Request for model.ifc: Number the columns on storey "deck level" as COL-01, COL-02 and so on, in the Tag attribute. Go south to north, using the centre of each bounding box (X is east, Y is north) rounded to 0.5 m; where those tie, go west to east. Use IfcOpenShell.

First a look at what the model holds.

```python
import ifcopenshell
import ifcopenshell.util.element
import ifcopenshell.util.placement

model = ifcopenshell.open("model.ifc")
print(model.schema)
storey = next(s for s in model.by_type("IfcBuildingStorey") if s.Name == "deck level")
columns = [e for e in ifcopenshell.util.element.get_decomposition(storey) if e.is_a("IfcColumn")]
for e in sorted(columns, key=lambda e: e.id()):
    origin = ifcopenshell.util.placement.get_local_placement(e.ObjectPlacement)[:3, 3]
    print(e.id(), e.Tag, e.Name, origin.round(2) + 0.0, sep=" | ")
```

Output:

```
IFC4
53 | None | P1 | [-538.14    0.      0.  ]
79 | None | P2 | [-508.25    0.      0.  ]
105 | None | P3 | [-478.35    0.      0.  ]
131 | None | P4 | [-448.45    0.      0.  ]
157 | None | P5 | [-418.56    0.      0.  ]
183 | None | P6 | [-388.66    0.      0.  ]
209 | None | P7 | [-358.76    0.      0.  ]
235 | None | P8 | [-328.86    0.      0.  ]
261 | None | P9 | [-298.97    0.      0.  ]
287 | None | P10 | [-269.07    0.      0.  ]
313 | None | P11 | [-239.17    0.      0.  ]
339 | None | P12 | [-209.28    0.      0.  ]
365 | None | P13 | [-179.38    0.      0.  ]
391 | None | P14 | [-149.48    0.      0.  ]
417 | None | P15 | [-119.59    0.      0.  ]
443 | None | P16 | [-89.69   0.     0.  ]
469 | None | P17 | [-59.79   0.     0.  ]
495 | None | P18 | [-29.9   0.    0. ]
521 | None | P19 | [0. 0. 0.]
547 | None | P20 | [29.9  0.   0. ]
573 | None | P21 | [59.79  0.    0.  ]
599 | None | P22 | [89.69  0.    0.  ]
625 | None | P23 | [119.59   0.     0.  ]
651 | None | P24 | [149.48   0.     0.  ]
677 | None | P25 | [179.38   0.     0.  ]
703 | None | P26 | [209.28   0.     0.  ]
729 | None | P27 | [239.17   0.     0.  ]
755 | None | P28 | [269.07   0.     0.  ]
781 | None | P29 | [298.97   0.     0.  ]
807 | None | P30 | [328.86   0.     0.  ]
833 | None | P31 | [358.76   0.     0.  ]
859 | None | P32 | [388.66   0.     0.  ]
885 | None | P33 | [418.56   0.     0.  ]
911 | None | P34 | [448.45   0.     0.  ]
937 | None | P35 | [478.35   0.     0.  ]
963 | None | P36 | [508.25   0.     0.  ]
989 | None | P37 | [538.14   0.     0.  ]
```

```python
import ifcopenshell
import ifcopenshell.geom
import ifcopenshell.util.element
import ifcopenshell.util.shape

model = ifcopenshell.open("model.ifc")
settings = ifcopenshell.geom.settings()
settings.set("use-world-coords", True)


def centre(element):
    shape = ifcopenshell.geom.create_shape(settings, element)
    return ifcopenshell.util.shape.get_bbox_centroid(shape.geometry)


storey = next(s for s in model.by_type("IfcBuildingStorey") if s.Name == "deck level")
columns = [e for e in ifcopenshell.util.element.get_decomposition(storey) if e.is_a("IfcColumn")]

# Insertion points can sit at a corner or the storey origin, so sort by the geometry (in metres).
centres = {e: centre(e) for e in columns}
columns.sort(key=lambda e: (round(centres[e][1] / 0.5), centres[e][0]))

for i, e in enumerate(columns, start=1):
    number = f"COL-{i:02d}"
    e.Tag = number
    print(e.id(), number)

model.write("model_rev.ifc")
```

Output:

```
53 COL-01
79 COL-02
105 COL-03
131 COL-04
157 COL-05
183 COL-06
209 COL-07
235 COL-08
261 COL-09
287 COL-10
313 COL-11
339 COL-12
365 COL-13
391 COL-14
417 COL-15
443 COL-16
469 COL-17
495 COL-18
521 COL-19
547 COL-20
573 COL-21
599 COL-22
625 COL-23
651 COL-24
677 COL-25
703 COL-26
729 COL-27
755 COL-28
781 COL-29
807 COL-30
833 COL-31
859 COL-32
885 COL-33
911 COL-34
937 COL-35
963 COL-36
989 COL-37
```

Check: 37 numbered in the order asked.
